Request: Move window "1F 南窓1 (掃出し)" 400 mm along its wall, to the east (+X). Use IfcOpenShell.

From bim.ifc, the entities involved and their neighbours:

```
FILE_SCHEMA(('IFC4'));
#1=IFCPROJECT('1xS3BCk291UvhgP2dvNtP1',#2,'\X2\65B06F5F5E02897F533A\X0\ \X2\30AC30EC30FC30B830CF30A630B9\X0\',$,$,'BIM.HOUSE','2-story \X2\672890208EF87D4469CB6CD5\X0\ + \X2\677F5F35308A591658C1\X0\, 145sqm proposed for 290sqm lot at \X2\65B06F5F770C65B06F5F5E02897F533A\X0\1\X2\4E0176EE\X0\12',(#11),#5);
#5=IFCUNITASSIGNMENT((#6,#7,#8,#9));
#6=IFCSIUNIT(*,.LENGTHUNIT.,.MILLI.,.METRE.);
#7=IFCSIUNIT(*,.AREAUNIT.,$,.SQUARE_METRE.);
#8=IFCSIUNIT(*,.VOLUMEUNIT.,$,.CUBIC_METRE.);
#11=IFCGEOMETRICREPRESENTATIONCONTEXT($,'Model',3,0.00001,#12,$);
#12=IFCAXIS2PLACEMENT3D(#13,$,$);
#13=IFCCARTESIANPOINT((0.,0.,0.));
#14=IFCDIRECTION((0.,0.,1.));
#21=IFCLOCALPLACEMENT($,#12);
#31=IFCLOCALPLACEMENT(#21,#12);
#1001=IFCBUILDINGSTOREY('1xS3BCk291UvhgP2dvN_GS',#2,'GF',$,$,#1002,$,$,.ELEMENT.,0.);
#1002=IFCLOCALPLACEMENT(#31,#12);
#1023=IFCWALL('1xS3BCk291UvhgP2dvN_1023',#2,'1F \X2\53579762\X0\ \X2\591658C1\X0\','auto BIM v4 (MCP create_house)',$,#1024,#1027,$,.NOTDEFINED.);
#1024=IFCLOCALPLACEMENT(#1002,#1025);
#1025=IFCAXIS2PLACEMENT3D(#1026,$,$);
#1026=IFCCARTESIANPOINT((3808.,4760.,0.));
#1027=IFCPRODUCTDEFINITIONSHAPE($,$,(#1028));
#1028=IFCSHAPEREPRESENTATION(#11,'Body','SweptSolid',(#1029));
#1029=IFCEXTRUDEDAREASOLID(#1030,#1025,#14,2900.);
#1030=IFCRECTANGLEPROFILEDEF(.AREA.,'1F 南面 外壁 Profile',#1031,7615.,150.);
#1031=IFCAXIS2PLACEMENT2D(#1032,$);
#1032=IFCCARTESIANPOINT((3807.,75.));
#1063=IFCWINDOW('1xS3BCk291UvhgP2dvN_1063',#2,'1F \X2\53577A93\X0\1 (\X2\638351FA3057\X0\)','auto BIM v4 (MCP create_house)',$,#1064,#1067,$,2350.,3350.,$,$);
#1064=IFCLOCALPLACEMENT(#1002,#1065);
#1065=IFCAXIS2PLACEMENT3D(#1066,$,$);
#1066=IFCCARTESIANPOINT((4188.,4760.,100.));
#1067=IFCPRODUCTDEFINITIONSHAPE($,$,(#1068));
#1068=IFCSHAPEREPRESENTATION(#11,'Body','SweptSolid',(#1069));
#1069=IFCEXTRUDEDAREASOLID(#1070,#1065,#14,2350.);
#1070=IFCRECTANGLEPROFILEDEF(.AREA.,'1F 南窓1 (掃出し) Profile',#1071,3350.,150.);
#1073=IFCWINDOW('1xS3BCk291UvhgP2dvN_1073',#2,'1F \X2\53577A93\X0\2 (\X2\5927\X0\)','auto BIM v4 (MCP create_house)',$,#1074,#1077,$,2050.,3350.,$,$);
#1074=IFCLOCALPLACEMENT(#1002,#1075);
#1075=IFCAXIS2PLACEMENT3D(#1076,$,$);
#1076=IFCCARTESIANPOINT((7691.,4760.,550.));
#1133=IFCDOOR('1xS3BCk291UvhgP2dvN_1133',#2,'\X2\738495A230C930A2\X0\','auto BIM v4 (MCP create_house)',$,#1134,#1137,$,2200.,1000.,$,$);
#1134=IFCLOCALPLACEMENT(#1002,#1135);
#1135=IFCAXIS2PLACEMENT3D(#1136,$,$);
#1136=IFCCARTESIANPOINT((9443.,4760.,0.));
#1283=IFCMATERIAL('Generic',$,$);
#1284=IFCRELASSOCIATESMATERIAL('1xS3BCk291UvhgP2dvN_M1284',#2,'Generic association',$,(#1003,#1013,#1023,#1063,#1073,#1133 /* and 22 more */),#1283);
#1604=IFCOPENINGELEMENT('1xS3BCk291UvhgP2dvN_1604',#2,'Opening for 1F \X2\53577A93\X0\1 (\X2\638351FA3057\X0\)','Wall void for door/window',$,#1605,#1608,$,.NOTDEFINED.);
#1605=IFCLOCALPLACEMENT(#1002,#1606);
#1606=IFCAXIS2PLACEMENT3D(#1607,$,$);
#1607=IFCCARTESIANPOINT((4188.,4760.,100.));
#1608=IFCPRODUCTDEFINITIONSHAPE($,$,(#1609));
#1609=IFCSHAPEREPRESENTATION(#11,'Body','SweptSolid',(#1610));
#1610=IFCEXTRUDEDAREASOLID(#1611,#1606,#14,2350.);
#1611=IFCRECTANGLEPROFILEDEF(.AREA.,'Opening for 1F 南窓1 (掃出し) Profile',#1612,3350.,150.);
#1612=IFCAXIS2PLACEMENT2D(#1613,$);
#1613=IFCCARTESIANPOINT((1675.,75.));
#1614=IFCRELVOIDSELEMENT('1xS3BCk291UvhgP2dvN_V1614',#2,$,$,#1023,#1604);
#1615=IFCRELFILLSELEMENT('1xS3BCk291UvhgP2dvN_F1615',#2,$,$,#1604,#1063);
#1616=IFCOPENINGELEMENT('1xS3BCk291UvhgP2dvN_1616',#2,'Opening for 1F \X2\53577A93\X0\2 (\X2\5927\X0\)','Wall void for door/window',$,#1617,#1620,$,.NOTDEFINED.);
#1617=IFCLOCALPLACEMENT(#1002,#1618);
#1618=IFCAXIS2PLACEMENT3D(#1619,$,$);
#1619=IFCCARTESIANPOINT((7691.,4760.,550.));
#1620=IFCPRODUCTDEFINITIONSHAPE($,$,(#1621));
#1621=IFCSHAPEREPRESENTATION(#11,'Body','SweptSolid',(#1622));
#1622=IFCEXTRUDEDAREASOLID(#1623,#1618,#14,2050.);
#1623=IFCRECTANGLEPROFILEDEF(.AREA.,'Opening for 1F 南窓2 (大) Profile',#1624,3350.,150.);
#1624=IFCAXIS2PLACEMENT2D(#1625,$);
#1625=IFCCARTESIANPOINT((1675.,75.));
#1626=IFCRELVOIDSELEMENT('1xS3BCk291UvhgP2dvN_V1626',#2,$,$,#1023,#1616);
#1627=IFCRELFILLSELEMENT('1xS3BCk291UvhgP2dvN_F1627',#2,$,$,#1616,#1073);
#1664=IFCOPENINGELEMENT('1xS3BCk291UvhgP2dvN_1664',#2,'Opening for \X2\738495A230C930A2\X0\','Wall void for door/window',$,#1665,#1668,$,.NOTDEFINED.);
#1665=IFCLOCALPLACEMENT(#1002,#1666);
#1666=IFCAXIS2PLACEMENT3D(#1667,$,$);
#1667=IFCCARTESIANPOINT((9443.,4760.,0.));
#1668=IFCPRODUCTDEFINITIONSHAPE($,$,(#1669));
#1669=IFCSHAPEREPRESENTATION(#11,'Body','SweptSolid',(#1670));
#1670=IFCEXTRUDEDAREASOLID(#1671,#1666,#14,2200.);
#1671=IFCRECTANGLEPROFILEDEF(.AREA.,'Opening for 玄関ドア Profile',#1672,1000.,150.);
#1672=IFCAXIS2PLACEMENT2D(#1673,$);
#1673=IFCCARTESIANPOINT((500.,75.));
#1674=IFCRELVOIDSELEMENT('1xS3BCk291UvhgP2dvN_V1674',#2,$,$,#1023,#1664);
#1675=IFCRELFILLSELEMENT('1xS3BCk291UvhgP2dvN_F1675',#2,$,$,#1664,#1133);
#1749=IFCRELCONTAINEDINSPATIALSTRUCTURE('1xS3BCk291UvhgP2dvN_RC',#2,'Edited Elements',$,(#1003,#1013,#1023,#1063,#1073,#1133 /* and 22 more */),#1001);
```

```python
import ifcopenshell
import ifcopenshell.api.geometry
import ifcopenshell.util.placement
import ifcopenshell.util.unit

model = ifcopenshell.open("bim.ifc")
unit_scale = ifcopenshell.util.unit.calculate_unit_scale(model)

window = model.by_id(1063)
opening = window.FillsVoids[0].RelatingOpeningElement
wall = opening.VoidsElements[0].RelatingBuildingElement

wall_matrix = ifcopenshell.util.placement.get_local_placement(wall.ObjectPlacement)
shift = wall_matrix[:3, 0] * 0.4 / unit_scale
before = ifcopenshell.util.placement.get_local_placement(window.ObjectPlacement)[:3, 3].copy()

# The window is not placed relative to its opening, so move both.
for product in (opening, window):
    matrix = ifcopenshell.util.placement.get_local_placement(product.ObjectPlacement)
    matrix[:3, 3] += shift
    ifcopenshell.api.geometry.edit_object_placement(model, product=product, matrix=matrix, is_si=False)

after = ifcopenshell.util.placement.get_local_placement(window.ObjectPlacement)[:3, 3]
print("window moved by", (after - before).round(3) + 0.0)

model.write("bim_edited.ifc")
```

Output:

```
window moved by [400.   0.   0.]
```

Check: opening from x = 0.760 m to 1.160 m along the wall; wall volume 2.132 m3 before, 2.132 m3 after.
